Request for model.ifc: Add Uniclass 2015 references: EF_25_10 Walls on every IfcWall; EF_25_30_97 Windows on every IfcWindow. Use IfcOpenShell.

First a look at what the model holds.

```python
import ifcopenshell

model = ifcopenshell.open("model.ifc")
print(model.schema)
print("classifications:", [c.Name for c in model.by_type("IfcClassification")])
for ifc_class in ("IfcDoor", "IfcRoof", "IfcStair", "IfcWall", "IfcWindow"):
    print(ifc_class, len(model.by_type(ifc_class)))
```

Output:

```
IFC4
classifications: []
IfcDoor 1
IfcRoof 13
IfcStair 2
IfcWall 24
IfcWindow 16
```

```python
import ifcopenshell
import ifcopenshell.api.classification

model = ifcopenshell.open("model.ifc")

system = ifcopenshell.api.classification.add_classification(model, classification="Uniclass 2015")

codes = {
    "IfcWall": ("EF_25_10", "Walls"),
    "IfcWindow": ("EF_25_30_97", "Windows"),
}
for ifc_class, (code, name) in codes.items():
    products = model.by_type(ifc_class)
    ifcopenshell.api.classification.add_reference(
        model, products=products, classification=system, identification=code, name=name
    )
    print(code, len(products))

model.write("model_v2.ifc")
```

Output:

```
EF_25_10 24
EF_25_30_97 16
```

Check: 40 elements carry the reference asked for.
